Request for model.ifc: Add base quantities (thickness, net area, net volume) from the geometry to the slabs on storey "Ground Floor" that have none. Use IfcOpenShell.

First a look at what the model holds.

```python
import ifcopenshell
import ifcopenshell.util.element
import ifcopenshell.util.unit

model = ifcopenshell.open("model.ifc")
print(model.schema)
for unit_type in ("LENGTHUNIT", "AREAUNIT", "VOLUMEUNIT"):
    print(unit_type, ifcopenshell.util.unit.calculate_unit_scale(model, unit_type))
storey = next(s for s in model.by_type("IfcBuildingStorey") if s.Name == "Ground Floor")
slabs = [e for e in ifcopenshell.util.element.get_decomposition(storey) if e.is_a("IfcSlab")]
for e in sorted(slabs, key=lambda e: e.id()):
    print(e.id(), e.is_a(), e.Name, list(ifcopenshell.util.element.get_psets(e, qtos_only=True)), sep=" | ")
```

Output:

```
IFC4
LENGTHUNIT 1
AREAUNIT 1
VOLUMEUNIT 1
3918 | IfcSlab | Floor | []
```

```python
import ifcopenshell
import ifcopenshell.api.pset
import ifcopenshell.geom
import ifcopenshell.util.element
import ifcopenshell.util.shape
import ifcopenshell.util.unit

model = ifcopenshell.open("model.ifc")
unit_scale = ifcopenshell.util.unit.calculate_unit_scale(model)
area_scale = ifcopenshell.util.unit.calculate_unit_scale(model, "AREAUNIT")
volume_scale = ifcopenshell.util.unit.calculate_unit_scale(model, "VOLUMEUNIT")
settings = ifcopenshell.geom.settings()

storey = next(s for s in model.by_type("IfcBuildingStorey") if s.Name == "Ground Floor")
slabs = [e for e in ifcopenshell.util.element.get_decomposition(storey) if e.is_a("IfcSlab")]

for e in sorted(slabs, key=lambda e: e.id()):
    if ifcopenshell.util.element.get_psets(e, qtos_only=True, should_inherit=False):
        continue
    # Geometry comes back in metres, in the element's own axes.
    shape = ifcopenshell.geom.create_shape(settings, e)
    values = {
        "Width": ifcopenshell.util.shape.get_z(shape.geometry) / unit_scale,
        "NetArea": ifcopenshell.util.shape.get_footprint_area(shape.geometry) / area_scale,
        "NetVolume": ifcopenshell.util.shape.get_volume(shape.geometry) / volume_scale,
    }
    qto = ifcopenshell.api.pset.add_qto(model, product=e, name="Qto_SlabBaseQuantities")
    ifcopenshell.api.pset.edit_qto(model, qto=qto, properties=values)
    print(e.id(), {k: round(v, 3) for k, v in values.items()})

model.write("model_edited.ifc")
```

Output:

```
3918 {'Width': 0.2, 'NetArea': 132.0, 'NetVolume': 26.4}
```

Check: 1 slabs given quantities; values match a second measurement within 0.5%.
